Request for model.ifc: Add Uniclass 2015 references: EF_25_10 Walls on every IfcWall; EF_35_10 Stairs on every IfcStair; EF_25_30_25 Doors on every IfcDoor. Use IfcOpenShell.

First a look at what the model holds.

```python
import ifcopenshell

model = ifcopenshell.open("model.ifc")
print(model.schema)
print("classifications:", [c.Name for c in model.by_type("IfcClassification")])
for ifc_class in ("IfcDoor", "IfcRoof", "IfcStair", "IfcWall", "IfcWindow"):
    print(ifc_class, len(model.by_type(ifc_class)))
```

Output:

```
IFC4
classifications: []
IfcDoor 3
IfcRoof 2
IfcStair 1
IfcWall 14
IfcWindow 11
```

```python
import ifcopenshell
import ifcopenshell.api.classification

model = ifcopenshell.open("model.ifc")

system = ifcopenshell.api.classification.add_classification(model, classification="Uniclass 2015")

codes = {
    "IfcWall": ("EF_25_10", "Walls"),
    "IfcStair": ("EF_35_10", "Stairs"),
    "IfcDoor": ("EF_25_30_25", "Doors"),
}
for ifc_class, (code, name) in codes.items():
    products = model.by_type(ifc_class)
    ifcopenshell.api.classification.add_reference(
        model, products=products, classification=system, identification=code, name=name
    )
    print(code, len(products))

model.write("model_rev.ifc")
```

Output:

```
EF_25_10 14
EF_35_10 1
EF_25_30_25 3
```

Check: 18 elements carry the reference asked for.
